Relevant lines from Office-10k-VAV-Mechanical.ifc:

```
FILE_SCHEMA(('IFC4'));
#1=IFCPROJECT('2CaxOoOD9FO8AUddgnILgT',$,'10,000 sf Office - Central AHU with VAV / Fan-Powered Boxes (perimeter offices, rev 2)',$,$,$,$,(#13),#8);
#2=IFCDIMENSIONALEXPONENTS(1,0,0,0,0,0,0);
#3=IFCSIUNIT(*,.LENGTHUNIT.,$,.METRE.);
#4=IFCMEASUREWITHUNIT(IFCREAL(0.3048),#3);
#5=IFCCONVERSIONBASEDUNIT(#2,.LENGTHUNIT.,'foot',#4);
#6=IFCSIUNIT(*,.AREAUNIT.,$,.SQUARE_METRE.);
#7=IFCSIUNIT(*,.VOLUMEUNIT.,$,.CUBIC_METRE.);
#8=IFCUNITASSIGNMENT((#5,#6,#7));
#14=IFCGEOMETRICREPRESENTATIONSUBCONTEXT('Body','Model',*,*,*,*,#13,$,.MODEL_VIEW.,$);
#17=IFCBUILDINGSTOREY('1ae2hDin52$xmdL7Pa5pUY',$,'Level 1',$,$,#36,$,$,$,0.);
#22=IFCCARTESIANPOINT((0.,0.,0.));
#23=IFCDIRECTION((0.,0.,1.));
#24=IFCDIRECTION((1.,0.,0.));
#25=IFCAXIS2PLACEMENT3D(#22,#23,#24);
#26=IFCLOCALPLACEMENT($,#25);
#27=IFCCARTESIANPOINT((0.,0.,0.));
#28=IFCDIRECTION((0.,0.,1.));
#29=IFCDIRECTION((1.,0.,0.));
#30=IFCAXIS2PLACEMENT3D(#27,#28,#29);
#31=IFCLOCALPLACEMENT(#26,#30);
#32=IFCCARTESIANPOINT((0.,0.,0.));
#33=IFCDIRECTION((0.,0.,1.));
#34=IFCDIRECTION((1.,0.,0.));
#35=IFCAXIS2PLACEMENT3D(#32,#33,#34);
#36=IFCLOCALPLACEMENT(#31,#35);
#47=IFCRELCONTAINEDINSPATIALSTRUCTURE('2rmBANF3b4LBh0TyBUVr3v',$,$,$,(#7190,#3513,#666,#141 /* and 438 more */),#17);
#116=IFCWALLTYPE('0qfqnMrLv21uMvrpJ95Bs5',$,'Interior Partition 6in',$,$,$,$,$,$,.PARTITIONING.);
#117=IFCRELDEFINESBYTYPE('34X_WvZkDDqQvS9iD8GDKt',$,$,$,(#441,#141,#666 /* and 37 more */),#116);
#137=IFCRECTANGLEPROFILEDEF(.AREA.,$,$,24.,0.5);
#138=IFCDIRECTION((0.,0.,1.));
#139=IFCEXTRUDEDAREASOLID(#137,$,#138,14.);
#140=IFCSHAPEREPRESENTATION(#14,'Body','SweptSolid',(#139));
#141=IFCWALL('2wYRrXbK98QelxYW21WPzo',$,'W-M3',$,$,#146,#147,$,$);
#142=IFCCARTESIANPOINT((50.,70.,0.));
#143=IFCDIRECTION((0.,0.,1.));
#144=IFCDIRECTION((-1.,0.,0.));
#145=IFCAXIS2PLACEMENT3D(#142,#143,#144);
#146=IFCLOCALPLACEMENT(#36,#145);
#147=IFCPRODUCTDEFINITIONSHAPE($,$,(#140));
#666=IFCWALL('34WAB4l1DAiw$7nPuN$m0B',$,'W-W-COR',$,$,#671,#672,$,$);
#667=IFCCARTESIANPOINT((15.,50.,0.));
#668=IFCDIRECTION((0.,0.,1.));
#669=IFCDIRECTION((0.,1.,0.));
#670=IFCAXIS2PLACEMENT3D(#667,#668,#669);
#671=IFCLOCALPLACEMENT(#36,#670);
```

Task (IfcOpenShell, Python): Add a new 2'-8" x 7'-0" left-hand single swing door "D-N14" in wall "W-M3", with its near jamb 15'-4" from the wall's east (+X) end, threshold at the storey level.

```python
import numpy as np
import ifcopenshell
import ifcopenshell.api.feature
import ifcopenshell.api.geometry
import ifcopenshell.api.root
import ifcopenshell.api.spatial
import ifcopenshell.geom
import ifcopenshell.util.element
import ifcopenshell.util.placement
import ifcopenshell.util.representation
import ifcopenshell.util.shape
import ifcopenshell.util.unit

model = ifcopenshell.open("Office-10k-VAV-Mechanical.ifc")
unit_scale = ifcopenshell.util.unit.calculate_unit_scale(model)
settings = ifcopenshell.geom.settings()


def volume(element):
    """Net volume in cubic metres, openings subtracted."""
    shape = ifcopenshell.geom.create_shape(settings, element)
    return ifcopenshell.util.shape.get_volume(shape.geometry)


wall = model.by_guid("2wYRrXbK98QelxYW21WPzo")
storey = ifcopenshell.util.element.get_container(wall, ifc_class="IfcBuildingStorey")
context = ifcopenshell.util.representation.get_context(model, "Model", "Body", "MODEL_VIEW")
before = volume(wall)

width, height, from_end, sill = 0.8128, 2.1336, 4.6736, 0.0  # metres

# The wall runs along its own X axis, and the end named is its -X end.
wall_shape = ifcopenshell.geom.create_shape(settings, wall)
x, y, z = ifcopenshell.util.shape.get_vertices(wall_shape.geometry).T
start = x.min() + from_end
face, thickness = float(y.min()), float(y.max() - y.min())
wall_matrix = ifcopenshell.util.placement.get_local_placement(wall.ObjectPlacement)
level = ifcopenshell.util.placement.get_local_placement(storey.ObjectPlacement)[2, 3]


def in_wall(x, y):
    """Placement at x, y metres in the wall's axes, at sill height."""
    matrix = wall_matrix.copy()
    matrix[:, 3] = wall_matrix @ np.array([x / unit_scale, y / unit_scale, 0.0, 1.0])
    matrix[2, 3] = level + sill / unit_scale
    return matrix


# Opening: a box that overshoots both wall faces by 50 mm.
opening = ifcopenshell.api.root.create_entity(model, ifc_class="IfcOpeningElement", predefined_type="OPENING")
box = ifcopenshell.api.geometry.add_wall_representation(
    model, context=context, length=width, height=height, thickness=thickness + 0.1
)
ifcopenshell.api.geometry.assign_representation(model, product=opening, representation=box)
ifcopenshell.api.geometry.edit_object_placement(model, product=opening, matrix=in_wall(start, face - 0.05), is_si=False)
ifcopenshell.api.feature.add_feature(model, feature=opening, element=wall)

door = ifcopenshell.api.root.create_entity(model, ifc_class="IfcDoor", name="D-N14", predefined_type="DOOR")
door.OverallWidth, door.OverallHeight = width / unit_scale, height / unit_scale
door.OperationType = "SINGLE_SWING_LEFT"
body = ifcopenshell.api.geometry.add_door_representation(
    model,
    context=context,
    overall_width=door.OverallWidth,
    overall_height=door.OverallHeight,
    operation_type="SINGLE_SWING_LEFT",
    lining_properties={"LiningDepth": thickness / unit_scale, "ThresholdDepth": thickness / unit_scale},
)
ifcopenshell.api.geometry.assign_representation(model, product=door, representation=body)
ifcopenshell.api.spatial.assign_container(model, products=[door], relating_structure=storey)
ifcopenshell.api.feature.add_filling(model, opening=opening, element=door)

# The lining spans the wall, so the door starts at the wall face.
ifcopenshell.api.geometry.edit_object_placement(model, product=door, matrix=in_wall(start, face), is_si=False)

after = volume(wall)

print(f"wall volume {before:.3f} -> {after:.3f} m3")

model.write("Office-10k-VAV-Mechanical_updated.ifc")
```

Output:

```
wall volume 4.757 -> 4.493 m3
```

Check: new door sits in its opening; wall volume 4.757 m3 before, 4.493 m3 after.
